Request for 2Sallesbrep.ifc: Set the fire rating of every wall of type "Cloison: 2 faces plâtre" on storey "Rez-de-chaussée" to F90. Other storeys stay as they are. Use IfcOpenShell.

First a look at what the model holds.

```python
import ifcopenshell
import ifcopenshell.util.element

model = ifcopenshell.open("2Sallesbrep.ifc")
print(model.schema)
storey = next(s for s in model.by_type("IfcBuildingStorey") if s.Name == "Rez-de-chaussée")
walls = [e for e in ifcopenshell.util.element.get_decomposition(storey) if e.is_a("IfcWall")]
seen = {}
for e in walls:
    element_type = ifcopenshell.util.element.get_type(e)
    key = (element_type.Name if element_type != e and element_type else None, ifcopenshell.util.element.get_pset(e, "Pset_WallCommon", "FireRating"))
    seen[key] = seen.get(key, 0) + 1
for (name, value), count in sorted(seen.items(), key=str):
    print(count, "x", name, "|", value)
```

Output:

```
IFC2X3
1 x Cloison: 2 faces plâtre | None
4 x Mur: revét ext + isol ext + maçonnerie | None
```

```python
import ifcopenshell
import ifcopenshell.api.pset
import ifcopenshell.util.element

model = ifcopenshell.open("2Sallesbrep.ifc")

storey = next(s for s in model.by_type("IfcBuildingStorey") if s.Name == "Rez-de-chaussée")
walls = [e for e in ifcopenshell.util.element.get_decomposition(storey) if e.is_a("IfcWall")]

count = 0
for e in walls:
    element_type = ifcopenshell.util.element.get_type(e)
    if element_type in (None, e) or element_type.Name != "Cloison: 2 faces plâtre":
        continue
    # add_pset returns the element's existing set when there is one.
    pset = ifcopenshell.api.pset.add_pset(model, product=e, name="Pset_WallCommon")
    ifcopenshell.api.pset.edit_pset(model, pset=pset, properties={"FireRating": "F90"})
    count += 1

print(count, "walls updated")

model.write("2Sallesbrep_rev.ifc")
```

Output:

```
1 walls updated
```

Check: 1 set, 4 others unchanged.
